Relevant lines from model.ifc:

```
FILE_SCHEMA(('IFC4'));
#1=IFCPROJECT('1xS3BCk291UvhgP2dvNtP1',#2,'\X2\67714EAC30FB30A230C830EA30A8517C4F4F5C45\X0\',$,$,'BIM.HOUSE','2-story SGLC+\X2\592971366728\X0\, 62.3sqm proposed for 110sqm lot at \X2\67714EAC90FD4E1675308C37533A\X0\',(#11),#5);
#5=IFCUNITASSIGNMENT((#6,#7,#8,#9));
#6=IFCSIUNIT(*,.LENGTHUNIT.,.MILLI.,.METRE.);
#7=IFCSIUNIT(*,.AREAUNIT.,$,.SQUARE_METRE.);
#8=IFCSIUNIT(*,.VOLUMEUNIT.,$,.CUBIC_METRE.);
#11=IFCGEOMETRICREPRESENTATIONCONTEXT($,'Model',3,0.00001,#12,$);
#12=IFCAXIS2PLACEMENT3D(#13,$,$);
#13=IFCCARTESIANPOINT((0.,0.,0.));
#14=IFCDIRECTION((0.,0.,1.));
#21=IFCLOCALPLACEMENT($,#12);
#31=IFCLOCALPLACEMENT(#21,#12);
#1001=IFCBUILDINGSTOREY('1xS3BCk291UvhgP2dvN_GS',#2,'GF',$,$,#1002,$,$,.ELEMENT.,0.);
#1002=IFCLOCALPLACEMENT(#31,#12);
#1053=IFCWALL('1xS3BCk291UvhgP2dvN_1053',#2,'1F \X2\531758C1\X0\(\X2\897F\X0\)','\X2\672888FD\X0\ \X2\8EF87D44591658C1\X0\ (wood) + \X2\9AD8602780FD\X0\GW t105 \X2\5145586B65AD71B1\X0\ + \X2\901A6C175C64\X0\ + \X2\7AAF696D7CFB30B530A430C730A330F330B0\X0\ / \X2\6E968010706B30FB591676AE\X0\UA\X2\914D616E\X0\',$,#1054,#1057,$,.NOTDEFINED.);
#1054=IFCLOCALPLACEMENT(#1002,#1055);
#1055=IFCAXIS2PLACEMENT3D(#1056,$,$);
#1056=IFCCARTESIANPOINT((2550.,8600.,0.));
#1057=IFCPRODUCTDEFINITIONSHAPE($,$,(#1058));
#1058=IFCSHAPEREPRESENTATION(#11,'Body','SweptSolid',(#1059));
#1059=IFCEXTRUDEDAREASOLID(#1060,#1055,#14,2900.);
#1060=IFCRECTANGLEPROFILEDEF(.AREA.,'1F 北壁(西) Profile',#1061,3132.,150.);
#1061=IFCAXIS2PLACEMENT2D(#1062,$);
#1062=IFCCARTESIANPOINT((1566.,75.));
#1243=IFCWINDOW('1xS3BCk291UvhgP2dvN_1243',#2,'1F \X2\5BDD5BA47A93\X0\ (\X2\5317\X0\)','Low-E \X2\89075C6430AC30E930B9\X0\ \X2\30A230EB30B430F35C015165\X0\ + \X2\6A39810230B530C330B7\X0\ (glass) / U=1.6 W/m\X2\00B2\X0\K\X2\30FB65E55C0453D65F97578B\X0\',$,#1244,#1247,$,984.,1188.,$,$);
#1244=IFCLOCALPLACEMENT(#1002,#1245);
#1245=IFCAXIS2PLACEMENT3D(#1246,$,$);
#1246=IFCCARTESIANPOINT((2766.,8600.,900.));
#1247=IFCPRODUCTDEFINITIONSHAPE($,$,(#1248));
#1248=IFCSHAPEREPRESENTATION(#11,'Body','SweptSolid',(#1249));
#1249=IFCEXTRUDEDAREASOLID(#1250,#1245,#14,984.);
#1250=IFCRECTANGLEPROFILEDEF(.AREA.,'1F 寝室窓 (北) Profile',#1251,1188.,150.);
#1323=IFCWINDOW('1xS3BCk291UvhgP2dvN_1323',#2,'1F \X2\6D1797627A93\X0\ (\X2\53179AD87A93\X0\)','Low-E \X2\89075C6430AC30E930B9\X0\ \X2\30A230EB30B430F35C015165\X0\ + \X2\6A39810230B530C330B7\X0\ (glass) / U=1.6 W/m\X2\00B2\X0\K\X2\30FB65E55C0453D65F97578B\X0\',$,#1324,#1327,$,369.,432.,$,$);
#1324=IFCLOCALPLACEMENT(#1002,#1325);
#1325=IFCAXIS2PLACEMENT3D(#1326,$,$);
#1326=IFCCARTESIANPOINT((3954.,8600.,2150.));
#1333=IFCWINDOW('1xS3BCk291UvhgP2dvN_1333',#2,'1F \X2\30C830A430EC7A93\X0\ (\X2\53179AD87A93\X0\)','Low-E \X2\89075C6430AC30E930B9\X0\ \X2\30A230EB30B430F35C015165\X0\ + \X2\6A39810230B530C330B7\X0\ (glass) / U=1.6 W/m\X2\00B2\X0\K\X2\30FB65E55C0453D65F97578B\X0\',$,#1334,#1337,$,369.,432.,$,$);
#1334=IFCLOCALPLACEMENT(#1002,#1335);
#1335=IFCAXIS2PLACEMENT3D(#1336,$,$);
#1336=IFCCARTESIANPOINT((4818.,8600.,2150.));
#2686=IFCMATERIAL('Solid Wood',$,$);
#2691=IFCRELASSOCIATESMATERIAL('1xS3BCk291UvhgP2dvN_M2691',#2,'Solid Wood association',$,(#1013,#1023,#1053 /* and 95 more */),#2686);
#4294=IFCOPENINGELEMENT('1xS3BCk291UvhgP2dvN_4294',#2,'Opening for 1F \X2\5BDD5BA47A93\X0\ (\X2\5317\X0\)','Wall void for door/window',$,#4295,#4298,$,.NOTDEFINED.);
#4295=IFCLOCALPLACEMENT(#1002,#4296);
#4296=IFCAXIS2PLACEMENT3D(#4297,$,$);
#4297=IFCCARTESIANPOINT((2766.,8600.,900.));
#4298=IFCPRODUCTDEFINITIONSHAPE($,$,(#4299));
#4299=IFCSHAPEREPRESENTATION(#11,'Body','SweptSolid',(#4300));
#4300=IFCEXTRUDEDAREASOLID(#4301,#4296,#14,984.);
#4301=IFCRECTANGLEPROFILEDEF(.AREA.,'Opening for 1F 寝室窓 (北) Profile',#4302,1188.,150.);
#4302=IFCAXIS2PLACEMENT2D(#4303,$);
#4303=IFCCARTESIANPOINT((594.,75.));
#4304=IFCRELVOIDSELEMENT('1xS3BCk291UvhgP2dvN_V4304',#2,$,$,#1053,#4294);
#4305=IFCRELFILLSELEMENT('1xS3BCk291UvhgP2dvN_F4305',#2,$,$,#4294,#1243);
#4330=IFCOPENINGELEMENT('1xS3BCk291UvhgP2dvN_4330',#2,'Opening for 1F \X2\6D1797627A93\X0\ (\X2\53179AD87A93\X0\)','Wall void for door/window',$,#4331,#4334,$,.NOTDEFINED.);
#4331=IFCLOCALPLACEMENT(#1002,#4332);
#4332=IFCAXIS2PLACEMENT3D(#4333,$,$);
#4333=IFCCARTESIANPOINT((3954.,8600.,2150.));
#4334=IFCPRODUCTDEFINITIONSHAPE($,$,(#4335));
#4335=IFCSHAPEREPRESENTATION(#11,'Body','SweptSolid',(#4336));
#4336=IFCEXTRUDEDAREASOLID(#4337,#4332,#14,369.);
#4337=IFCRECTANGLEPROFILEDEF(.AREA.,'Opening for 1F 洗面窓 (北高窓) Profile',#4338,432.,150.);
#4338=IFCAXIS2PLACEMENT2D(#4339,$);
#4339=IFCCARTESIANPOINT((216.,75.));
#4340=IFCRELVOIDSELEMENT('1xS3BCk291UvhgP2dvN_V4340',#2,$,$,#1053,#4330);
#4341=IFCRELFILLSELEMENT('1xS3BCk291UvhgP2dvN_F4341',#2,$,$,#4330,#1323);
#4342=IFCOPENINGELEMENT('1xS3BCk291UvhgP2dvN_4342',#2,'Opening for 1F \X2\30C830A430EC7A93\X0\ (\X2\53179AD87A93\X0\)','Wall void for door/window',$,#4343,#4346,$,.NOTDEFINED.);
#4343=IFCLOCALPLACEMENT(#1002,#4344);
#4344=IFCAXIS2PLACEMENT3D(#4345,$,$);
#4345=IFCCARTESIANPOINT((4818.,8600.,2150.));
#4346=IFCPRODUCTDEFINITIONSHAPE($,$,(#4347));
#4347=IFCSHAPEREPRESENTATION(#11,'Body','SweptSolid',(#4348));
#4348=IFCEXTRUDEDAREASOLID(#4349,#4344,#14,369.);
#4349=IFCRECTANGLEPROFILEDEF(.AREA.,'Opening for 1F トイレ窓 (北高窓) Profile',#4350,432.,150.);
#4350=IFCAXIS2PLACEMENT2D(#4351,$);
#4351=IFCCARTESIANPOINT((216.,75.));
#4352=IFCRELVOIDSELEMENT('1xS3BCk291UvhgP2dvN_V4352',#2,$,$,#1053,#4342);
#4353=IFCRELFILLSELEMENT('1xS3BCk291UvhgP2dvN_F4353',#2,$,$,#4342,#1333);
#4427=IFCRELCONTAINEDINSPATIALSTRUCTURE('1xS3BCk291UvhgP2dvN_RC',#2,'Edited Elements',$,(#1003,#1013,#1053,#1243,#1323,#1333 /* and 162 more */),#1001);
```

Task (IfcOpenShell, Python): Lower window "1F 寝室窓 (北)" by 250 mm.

```python
import numpy as np
import ifcopenshell
import ifcopenshell.api.geometry
import ifcopenshell.util.placement
import ifcopenshell.util.unit

model = ifcopenshell.open("model.ifc")
unit_scale = ifcopenshell.util.unit.calculate_unit_scale(model)

window = model.by_guid("1xS3BCk291UvhgP2dvN_1243")
opening = window.FillsVoids[0].RelatingOpeningElement
dz = -0.25 / unit_scale

shift = np.array([0.0, 0.0, dz])
# The window is not placed relative to its opening, so move both.
for product in (opening, window):
    matrix = ifcopenshell.util.placement.get_local_placement(product.ObjectPlacement)
    matrix[:3, 3] += shift
    ifcopenshell.api.geometry.edit_object_placement(model, product=product, matrix=matrix, is_si=False)

print(f"moved by {dz * unit_scale:+.3f} m")

model.write("model_updated.ifc")
```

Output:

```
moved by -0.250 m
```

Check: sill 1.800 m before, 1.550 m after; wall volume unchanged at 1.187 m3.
